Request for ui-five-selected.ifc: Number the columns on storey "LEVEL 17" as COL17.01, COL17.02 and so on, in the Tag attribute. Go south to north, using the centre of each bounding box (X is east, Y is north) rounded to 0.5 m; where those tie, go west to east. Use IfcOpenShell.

First a look at what the model holds.

```python
import ifcopenshell
import ifcopenshell.util.element
import ifcopenshell.util.placement

model = ifcopenshell.open("ui-five-selected.ifc")
print(model.schema)
storey = next(s for s in model.by_type("IfcBuildingStorey") if s.Name == "LEVEL 17")
columns = [e for e in ifcopenshell.util.element.get_decomposition(storey) if e.is_a("IfcColumn")]
for e in sorted(columns, key=lambda e: e.id()):
    origin = ifcopenshell.util.placement.get_local_placement(e.ObjectPlacement)[:3, 3]
    print(e.id(), e.Tag, e.Name, origin.round(2) + 0.0, sep=" | ")
```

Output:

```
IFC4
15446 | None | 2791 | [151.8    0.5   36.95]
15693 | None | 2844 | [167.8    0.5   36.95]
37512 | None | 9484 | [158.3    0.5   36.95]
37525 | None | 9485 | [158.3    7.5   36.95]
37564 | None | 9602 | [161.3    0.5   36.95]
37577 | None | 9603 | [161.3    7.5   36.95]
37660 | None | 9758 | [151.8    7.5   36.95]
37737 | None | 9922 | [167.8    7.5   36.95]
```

```python
import ifcopenshell
import ifcopenshell.geom
import ifcopenshell.util.element
import ifcopenshell.util.shape

model = ifcopenshell.open("ui-five-selected.ifc")
settings = ifcopenshell.geom.settings()
settings.set("use-world-coords", True)


def centre(element):
    shape = ifcopenshell.geom.create_shape(settings, element)
    return ifcopenshell.util.shape.get_bbox_centroid(shape.geometry)


storey = next(s for s in model.by_type("IfcBuildingStorey") if s.Name == "LEVEL 17")
columns = [e for e in ifcopenshell.util.element.get_decomposition(storey) if e.is_a("IfcColumn")]

# Insertion points can sit at a corner or the storey origin, so sort by the geometry (in metres).
centres = {e: centre(e) for e in columns}
columns.sort(key=lambda e: (round(centres[e][1] / 0.5), centres[e][0]))

for i, e in enumerate(columns, start=1):
    number = f"COL17.{i:02d}"
    e.Tag = number
    print(e.id(), number)

model.write("ui-five-selected_v2.ifc")
```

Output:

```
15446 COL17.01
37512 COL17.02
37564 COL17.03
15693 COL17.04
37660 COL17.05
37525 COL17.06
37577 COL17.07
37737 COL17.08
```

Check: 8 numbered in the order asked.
